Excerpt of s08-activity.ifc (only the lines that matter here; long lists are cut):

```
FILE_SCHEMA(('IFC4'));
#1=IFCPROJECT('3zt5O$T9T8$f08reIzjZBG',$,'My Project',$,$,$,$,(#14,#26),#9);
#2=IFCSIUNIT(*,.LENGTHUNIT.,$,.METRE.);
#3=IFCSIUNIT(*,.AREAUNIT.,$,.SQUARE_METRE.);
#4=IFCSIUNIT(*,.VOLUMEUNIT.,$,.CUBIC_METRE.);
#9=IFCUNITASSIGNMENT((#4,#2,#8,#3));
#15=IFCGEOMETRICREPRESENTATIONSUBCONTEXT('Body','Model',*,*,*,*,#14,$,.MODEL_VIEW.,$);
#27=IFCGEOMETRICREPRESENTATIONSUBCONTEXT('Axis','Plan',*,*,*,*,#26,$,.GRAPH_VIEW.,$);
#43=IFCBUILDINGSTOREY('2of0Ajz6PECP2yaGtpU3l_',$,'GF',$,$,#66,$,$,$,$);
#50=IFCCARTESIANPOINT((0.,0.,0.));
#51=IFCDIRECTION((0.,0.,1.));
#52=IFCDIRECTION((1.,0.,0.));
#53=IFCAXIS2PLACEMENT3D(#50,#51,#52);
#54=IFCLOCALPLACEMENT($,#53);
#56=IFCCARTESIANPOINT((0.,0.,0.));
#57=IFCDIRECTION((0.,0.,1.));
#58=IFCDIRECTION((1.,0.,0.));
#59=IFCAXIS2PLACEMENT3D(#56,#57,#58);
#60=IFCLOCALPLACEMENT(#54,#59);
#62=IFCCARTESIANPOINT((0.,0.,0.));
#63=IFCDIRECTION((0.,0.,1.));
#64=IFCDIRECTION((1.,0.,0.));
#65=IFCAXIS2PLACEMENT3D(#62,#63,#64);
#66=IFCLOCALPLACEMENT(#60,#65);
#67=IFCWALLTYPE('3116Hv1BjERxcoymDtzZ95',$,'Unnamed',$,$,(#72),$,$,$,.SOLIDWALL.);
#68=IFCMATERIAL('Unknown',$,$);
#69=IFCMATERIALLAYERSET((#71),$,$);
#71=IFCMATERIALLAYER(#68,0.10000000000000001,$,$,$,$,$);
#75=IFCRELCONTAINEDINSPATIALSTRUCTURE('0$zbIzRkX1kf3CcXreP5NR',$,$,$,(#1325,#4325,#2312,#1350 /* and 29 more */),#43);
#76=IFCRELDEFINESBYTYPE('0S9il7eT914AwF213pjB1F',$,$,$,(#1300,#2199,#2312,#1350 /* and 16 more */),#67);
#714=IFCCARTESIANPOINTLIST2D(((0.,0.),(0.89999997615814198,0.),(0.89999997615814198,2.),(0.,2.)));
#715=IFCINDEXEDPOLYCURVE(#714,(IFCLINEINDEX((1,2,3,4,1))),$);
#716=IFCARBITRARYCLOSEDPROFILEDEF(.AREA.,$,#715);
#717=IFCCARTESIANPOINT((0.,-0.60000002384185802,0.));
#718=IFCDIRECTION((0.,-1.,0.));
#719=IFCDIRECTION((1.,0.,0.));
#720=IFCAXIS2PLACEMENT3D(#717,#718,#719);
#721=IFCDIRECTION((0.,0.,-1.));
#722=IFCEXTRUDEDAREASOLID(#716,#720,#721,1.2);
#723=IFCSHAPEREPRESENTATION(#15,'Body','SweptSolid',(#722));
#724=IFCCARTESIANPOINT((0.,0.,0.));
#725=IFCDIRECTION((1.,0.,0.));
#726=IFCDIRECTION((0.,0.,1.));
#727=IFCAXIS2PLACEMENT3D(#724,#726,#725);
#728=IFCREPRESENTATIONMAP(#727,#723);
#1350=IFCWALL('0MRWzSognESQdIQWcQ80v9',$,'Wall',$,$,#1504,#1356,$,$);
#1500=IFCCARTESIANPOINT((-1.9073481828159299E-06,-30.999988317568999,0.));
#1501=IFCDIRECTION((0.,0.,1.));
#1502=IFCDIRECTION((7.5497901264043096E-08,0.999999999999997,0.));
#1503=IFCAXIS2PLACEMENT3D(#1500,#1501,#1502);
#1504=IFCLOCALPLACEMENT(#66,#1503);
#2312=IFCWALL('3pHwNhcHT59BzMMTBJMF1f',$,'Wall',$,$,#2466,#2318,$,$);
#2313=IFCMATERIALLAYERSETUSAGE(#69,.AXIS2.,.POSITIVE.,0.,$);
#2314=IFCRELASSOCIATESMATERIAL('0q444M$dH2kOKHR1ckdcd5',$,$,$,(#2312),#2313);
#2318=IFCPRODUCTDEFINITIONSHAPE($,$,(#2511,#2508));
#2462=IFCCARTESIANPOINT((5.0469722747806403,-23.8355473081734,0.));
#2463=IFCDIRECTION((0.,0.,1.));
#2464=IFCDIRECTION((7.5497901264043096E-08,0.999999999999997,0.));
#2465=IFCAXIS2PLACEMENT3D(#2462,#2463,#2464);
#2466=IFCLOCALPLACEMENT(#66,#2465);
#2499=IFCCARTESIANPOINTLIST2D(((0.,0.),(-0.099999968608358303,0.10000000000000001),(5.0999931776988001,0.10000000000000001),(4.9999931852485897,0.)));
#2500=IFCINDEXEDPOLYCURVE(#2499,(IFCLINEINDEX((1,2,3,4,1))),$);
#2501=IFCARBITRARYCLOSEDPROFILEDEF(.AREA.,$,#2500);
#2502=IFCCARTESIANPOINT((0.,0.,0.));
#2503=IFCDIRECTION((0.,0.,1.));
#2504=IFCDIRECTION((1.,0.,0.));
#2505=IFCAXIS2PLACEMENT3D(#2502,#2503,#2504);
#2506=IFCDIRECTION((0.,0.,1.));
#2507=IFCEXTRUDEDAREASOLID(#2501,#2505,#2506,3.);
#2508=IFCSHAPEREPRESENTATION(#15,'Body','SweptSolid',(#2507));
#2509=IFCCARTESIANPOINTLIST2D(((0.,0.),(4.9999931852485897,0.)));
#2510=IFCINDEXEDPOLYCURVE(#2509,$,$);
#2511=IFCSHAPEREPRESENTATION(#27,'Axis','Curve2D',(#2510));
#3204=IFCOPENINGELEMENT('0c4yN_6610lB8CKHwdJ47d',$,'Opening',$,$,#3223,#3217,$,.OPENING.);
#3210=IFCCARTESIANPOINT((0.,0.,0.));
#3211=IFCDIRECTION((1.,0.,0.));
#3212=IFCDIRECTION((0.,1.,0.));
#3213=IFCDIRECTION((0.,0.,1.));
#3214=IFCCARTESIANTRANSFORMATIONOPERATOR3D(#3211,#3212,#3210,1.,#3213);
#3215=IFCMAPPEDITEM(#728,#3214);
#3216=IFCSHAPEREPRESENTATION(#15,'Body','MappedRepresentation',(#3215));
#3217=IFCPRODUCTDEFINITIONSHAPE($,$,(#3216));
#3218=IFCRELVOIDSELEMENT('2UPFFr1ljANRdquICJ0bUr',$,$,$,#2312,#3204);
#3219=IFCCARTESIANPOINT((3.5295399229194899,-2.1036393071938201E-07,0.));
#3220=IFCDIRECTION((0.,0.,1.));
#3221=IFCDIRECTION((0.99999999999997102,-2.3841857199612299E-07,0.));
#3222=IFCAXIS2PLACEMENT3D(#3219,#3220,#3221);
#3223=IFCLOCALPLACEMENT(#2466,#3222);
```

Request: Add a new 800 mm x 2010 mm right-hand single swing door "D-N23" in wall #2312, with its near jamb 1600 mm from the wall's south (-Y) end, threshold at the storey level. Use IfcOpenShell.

```python
import numpy as np
import ifcopenshell
import ifcopenshell.api.feature
import ifcopenshell.api.geometry
import ifcopenshell.api.root
import ifcopenshell.api.spatial
import ifcopenshell.geom
import ifcopenshell.util.element
import ifcopenshell.util.placement
import ifcopenshell.util.representation
import ifcopenshell.util.shape
import ifcopenshell.util.unit

model = ifcopenshell.open("s08-activity.ifc")
unit_scale = ifcopenshell.util.unit.calculate_unit_scale(model)
settings = ifcopenshell.geom.settings()


def volume(element):
    """Net volume in cubic metres, openings subtracted."""
    shape = ifcopenshell.geom.create_shape(settings, element)
    return ifcopenshell.util.shape.get_volume(shape.geometry)


wall = model.by_guid("3pHwNhcHT59BzMMTBJMF1f")
storey = ifcopenshell.util.element.get_container(wall, ifc_class="IfcBuildingStorey")
context = ifcopenshell.util.representation.get_context(model, "Model", "Body", "MODEL_VIEW")
before = volume(wall)

width, height, from_end, sill = 0.8, 2.01, 1.6, 0.0  # metres

# The wall runs along its own X axis, and the end named is its -X end.
wall_shape = ifcopenshell.geom.create_shape(settings, wall)
x, y, z = ifcopenshell.util.shape.get_vertices(wall_shape.geometry).T
start = x.min() + from_end
face, thickness = float(y.min()), float(y.max() - y.min())
wall_matrix = ifcopenshell.util.placement.get_local_placement(wall.ObjectPlacement)
level = ifcopenshell.util.placement.get_local_placement(storey.ObjectPlacement)[2, 3]


def in_wall(x, y):
    """Placement at x, y metres in the wall's axes, at sill height."""
    matrix = wall_matrix.copy()
    matrix[:, 3] = wall_matrix @ np.array([x / unit_scale, y / unit_scale, 0.0, 1.0])
    matrix[2, 3] = level + sill / unit_scale
    return matrix


# Opening: a box that overshoots both wall faces by 50 mm.
opening = ifcopenshell.api.root.create_entity(model, ifc_class="IfcOpeningElement", predefined_type="OPENING")
box = ifcopenshell.api.geometry.add_wall_representation(
    model, context=context, length=width, height=height, thickness=thickness + 0.1
)
ifcopenshell.api.geometry.assign_representation(model, product=opening, representation=box)
ifcopenshell.api.geometry.edit_object_placement(model, product=opening, matrix=in_wall(start, face - 0.05), is_si=False)
ifcopenshell.api.feature.add_feature(model, feature=opening, element=wall)

door = ifcopenshell.api.root.create_entity(model, ifc_class="IfcDoor", name="D-N23", predefined_type="DOOR")
door.OverallWidth, door.OverallHeight = width / unit_scale, height / unit_scale
door.OperationType = "SINGLE_SWING_RIGHT"
body = ifcopenshell.api.geometry.add_door_representation(
    model,
    context=context,
    overall_width=door.OverallWidth,
    overall_height=door.OverallHeight,
    operation_type="SINGLE_SWING_RIGHT",
    lining_properties={"LiningDepth": thickness / unit_scale, "ThresholdDepth": thickness / unit_scale},
)
ifcopenshell.api.geometry.assign_representation(model, product=door, representation=body)
ifcopenshell.api.spatial.assign_container(model, products=[door], relating_structure=storey)
ifcopenshell.api.feature.add_filling(model, opening=opening, element=door)

# The lining spans the wall, so the door starts at the wall face.
ifcopenshell.api.geometry.edit_object_placement(model, product=door, matrix=in_wall(start, face), is_si=False)

after = volume(wall)

print(f"wall volume {before:.3f} -> {after:.3f} m3")

model.write("s08-activity-out.ifc")
```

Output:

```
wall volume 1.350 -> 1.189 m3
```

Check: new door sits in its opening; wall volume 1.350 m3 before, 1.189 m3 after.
